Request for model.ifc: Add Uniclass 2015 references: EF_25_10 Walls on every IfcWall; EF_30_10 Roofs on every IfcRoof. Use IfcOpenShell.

First a look at what the model holds.

```python
import ifcopenshell

model = ifcopenshell.open("model.ifc")
print(model.schema)
print("classifications:", [c.Name for c in model.by_type("IfcClassification")])
for ifc_class in ("IfcDoor", "IfcRoof", "IfcStair", "IfcWall", "IfcWindow"):
    print(ifc_class, len(model.by_type(ifc_class)))
```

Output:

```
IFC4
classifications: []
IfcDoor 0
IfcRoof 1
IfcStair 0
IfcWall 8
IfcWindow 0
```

```python
import ifcopenshell
import ifcopenshell.api.classification

model = ifcopenshell.open("model.ifc")

system = ifcopenshell.api.classification.add_classification(model, classification="Uniclass 2015")

codes = {
    "IfcWall": ("EF_25_10", "Walls"),
    "IfcRoof": ("EF_30_10", "Roofs"),
}
for ifc_class, (code, name) in codes.items():
    products = model.by_type(ifc_class)
    ifcopenshell.api.classification.add_reference(
        model, products=products, classification=system, identification=code, name=name
    )
    print(code, len(products))

model.write("model_updated.ifc")
```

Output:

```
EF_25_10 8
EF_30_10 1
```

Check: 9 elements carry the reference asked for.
